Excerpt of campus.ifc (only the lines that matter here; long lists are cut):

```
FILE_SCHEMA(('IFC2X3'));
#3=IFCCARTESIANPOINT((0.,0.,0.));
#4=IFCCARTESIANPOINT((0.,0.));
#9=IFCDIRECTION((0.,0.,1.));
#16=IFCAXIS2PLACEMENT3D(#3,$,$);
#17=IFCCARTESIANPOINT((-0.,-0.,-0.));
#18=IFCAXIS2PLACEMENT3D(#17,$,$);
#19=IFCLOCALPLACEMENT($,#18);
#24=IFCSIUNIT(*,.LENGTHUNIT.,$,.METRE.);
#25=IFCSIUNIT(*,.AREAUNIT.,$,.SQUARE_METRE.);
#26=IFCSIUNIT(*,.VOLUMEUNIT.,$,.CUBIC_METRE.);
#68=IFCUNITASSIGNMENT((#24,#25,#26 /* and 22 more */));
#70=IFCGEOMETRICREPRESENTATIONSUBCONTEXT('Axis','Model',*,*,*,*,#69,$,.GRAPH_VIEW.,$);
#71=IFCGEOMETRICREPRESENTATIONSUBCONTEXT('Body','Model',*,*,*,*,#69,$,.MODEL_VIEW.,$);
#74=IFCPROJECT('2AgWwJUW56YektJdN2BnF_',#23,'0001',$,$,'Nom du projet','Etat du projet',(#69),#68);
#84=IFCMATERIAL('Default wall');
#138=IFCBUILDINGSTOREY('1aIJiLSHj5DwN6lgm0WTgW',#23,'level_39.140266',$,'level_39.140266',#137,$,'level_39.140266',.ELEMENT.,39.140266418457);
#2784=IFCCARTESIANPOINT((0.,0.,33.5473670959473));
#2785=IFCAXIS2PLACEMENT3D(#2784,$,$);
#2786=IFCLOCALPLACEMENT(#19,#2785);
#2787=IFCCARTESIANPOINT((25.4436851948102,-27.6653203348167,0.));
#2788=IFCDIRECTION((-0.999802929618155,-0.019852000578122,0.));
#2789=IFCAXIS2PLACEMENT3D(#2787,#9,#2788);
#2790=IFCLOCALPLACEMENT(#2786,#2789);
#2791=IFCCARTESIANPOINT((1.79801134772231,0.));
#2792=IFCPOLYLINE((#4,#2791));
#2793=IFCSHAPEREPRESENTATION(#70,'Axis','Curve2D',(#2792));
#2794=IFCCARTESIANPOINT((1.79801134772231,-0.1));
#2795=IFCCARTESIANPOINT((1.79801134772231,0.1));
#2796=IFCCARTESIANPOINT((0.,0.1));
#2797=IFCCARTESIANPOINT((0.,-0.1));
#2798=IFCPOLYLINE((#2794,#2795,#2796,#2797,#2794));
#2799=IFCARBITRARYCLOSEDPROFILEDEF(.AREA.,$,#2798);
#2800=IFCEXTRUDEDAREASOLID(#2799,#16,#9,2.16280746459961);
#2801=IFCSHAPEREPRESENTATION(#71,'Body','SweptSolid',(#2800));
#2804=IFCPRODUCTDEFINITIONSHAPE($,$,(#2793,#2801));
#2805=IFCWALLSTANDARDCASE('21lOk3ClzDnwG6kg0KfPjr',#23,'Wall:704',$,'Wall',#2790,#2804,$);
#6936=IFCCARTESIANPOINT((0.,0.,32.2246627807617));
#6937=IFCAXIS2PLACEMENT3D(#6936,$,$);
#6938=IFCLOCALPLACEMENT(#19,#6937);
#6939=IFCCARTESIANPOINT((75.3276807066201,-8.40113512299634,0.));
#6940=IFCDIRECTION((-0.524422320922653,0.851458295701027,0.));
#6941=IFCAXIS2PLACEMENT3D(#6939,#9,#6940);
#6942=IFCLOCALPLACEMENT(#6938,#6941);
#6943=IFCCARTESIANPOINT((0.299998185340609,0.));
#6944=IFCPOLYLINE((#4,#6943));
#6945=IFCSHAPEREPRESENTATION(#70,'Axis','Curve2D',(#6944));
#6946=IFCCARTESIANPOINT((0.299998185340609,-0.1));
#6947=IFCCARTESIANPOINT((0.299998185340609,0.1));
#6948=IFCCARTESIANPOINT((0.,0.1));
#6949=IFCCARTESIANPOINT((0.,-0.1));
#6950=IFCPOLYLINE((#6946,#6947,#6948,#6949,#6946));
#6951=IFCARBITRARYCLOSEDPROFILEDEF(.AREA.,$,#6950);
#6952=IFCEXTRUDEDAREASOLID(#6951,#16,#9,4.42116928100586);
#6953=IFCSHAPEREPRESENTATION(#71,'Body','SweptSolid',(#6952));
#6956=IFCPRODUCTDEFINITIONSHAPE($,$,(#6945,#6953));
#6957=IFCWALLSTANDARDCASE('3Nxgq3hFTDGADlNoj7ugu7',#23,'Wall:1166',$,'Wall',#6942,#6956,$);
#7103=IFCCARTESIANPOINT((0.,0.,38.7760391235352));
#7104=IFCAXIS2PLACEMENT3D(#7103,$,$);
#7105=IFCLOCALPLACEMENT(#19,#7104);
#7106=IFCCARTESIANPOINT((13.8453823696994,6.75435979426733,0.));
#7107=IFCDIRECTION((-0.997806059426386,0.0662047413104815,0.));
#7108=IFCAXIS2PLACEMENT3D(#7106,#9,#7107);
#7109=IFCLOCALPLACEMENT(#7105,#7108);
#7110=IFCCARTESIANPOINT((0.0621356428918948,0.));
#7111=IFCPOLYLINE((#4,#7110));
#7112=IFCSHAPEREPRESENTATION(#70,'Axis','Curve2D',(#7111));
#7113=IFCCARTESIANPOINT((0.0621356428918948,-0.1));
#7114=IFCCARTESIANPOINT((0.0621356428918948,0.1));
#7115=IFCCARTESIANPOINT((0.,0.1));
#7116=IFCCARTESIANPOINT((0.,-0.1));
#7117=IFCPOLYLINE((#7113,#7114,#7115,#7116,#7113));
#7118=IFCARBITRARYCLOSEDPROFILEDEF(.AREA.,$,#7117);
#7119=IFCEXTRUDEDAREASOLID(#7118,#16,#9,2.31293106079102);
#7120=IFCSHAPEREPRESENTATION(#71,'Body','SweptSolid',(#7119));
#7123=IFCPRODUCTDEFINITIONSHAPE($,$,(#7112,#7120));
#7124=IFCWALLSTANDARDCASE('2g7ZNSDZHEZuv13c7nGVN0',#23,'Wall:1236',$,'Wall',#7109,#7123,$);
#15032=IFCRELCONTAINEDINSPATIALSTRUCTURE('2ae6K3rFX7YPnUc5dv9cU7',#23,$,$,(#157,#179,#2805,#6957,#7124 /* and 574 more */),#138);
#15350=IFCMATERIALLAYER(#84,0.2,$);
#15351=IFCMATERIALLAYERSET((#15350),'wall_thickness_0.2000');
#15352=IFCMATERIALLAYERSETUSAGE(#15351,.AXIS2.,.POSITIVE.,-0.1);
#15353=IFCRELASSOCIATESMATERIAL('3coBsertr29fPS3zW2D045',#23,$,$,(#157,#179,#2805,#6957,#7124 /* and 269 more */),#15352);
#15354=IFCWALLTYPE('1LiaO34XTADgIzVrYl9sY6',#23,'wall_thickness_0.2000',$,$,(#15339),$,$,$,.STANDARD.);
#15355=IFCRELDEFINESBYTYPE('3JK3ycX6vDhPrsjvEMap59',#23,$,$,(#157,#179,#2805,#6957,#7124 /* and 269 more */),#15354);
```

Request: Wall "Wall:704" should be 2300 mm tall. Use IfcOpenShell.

```python
import ifcopenshell
import ifcopenshell.geom
import ifcopenshell.util.representation
import ifcopenshell.util.shape
import ifcopenshell.util.unit

model = ifcopenshell.open("campus.ifc")
unit_scale = ifcopenshell.util.unit.calculate_unit_scale(model)
settings = ifcopenshell.geom.settings()


def volume(element):
    """Net volume in cubic metres, openings subtracted."""
    shape = ifcopenshell.geom.create_shape(settings, element)
    return ifcopenshell.util.shape.get_volume(shape.geometry)


wall = model.by_id(2805)
before = volume(wall)

body = ifcopenshell.util.representation.get_representation(wall, "Model", "Body")
solid = body.Items[0]
old_height = solid.Depth
solid.Depth = 2.3 / unit_scale
after = volume(wall)

print(f"height {old_height:g} -> {solid.Depth:g}, volume {before:.3f} -> {after:.3f} m3")

model.write("campus_edited.ifc")
```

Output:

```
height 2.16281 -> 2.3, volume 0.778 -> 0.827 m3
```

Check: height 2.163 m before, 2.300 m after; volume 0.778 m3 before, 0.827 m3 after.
